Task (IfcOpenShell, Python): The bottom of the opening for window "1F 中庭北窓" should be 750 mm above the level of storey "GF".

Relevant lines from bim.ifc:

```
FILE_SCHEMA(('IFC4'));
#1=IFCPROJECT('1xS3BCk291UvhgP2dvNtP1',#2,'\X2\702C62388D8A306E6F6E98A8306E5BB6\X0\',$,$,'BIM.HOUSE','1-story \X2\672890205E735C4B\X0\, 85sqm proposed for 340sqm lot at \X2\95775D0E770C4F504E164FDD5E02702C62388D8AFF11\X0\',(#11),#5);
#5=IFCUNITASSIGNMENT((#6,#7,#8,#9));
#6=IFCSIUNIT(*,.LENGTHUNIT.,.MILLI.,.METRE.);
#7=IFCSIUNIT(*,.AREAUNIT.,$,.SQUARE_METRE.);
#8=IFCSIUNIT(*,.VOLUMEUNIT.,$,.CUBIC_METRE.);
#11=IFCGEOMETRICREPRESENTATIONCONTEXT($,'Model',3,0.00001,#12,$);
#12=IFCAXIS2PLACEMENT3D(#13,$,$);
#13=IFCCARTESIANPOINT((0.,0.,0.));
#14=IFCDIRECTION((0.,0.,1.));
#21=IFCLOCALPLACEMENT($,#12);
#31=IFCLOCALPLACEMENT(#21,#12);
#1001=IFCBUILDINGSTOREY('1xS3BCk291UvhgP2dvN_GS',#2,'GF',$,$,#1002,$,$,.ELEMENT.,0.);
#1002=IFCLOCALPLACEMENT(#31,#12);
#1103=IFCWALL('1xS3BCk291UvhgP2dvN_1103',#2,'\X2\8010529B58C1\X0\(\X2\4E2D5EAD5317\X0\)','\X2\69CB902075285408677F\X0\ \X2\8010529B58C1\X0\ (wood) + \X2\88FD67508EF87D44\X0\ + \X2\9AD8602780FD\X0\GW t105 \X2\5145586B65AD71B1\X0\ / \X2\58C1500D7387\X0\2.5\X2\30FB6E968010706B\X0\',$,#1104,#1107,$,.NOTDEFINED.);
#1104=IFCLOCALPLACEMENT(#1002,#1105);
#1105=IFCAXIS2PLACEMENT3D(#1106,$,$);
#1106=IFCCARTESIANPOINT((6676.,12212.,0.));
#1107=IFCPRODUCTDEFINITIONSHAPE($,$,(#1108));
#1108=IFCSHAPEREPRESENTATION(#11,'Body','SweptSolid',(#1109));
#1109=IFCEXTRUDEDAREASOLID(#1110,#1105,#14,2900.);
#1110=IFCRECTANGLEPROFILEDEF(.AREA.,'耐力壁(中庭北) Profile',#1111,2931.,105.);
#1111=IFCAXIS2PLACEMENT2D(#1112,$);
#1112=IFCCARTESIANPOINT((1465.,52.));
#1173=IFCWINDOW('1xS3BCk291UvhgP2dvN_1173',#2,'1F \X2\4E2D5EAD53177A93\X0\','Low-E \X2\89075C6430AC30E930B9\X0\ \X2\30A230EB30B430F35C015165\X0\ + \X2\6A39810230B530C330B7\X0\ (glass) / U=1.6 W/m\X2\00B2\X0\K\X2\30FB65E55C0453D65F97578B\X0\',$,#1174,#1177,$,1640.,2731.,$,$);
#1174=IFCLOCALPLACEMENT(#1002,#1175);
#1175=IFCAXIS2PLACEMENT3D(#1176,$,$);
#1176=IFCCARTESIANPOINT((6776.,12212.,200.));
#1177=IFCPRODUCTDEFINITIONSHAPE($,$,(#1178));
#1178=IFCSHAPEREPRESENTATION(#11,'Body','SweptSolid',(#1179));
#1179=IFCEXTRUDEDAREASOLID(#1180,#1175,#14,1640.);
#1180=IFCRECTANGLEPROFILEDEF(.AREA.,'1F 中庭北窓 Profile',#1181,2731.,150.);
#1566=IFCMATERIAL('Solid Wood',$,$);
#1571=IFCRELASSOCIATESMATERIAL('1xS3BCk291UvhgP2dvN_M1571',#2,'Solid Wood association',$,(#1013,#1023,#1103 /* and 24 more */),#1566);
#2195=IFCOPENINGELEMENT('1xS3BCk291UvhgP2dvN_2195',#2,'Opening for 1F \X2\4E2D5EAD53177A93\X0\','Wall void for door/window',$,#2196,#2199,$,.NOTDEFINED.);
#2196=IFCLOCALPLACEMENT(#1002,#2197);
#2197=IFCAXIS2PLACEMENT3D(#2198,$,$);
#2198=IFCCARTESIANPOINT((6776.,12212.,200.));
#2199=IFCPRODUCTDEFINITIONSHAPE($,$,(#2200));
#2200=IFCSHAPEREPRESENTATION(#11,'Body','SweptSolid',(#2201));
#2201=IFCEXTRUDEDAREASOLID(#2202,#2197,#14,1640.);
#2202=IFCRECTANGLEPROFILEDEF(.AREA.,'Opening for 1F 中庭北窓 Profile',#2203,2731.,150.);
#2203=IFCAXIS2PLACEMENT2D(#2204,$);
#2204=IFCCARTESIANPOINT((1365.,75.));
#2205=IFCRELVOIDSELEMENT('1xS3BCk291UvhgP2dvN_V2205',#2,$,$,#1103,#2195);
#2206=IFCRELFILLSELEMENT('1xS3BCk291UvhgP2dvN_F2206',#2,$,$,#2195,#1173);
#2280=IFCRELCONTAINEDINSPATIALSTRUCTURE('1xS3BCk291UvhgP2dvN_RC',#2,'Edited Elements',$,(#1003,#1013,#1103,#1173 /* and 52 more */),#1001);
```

```python
import numpy as np
import ifcopenshell
import ifcopenshell.api.geometry
import ifcopenshell.geom
import ifcopenshell.util.element
import ifcopenshell.util.placement
import ifcopenshell.util.shape
import ifcopenshell.util.unit

model = ifcopenshell.open("bim.ifc")
unit_scale = ifcopenshell.util.unit.calculate_unit_scale(model)

window = model.by_guid("1xS3BCk291UvhgP2dvN_1173")
opening = window.FillsVoids[0].RelatingOpeningElement
storey = ifcopenshell.util.element.get_container(window, ifc_class="IfcBuildingStorey")
level = ifcopenshell.util.placement.get_local_placement(storey.ObjectPlacement)[2, 3]

# The opening's origin need not be at the sill, so measure its lowest point.
shape = ifcopenshell.geom.create_shape(ifcopenshell.geom.settings(), opening)
bottom = ifcopenshell.util.shape.get_shape_bottom_elevation(shape, shape.geometry) / unit_scale
dz = level + 750.0 - bottom

shift = np.array([0.0, 0.0, dz])
# The window is not placed relative to its opening, so move both.
for product in (opening, window):
    matrix = ifcopenshell.util.placement.get_local_placement(product.ObjectPlacement)
    matrix[:3, 3] += shift
    ifcopenshell.api.geometry.edit_object_placement(model, product=product, matrix=matrix, is_si=False)

print(f"moved by {dz * unit_scale:+.3f} m")

model.write("bim_v2.ifc")
```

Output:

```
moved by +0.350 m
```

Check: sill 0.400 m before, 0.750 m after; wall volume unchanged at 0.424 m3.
